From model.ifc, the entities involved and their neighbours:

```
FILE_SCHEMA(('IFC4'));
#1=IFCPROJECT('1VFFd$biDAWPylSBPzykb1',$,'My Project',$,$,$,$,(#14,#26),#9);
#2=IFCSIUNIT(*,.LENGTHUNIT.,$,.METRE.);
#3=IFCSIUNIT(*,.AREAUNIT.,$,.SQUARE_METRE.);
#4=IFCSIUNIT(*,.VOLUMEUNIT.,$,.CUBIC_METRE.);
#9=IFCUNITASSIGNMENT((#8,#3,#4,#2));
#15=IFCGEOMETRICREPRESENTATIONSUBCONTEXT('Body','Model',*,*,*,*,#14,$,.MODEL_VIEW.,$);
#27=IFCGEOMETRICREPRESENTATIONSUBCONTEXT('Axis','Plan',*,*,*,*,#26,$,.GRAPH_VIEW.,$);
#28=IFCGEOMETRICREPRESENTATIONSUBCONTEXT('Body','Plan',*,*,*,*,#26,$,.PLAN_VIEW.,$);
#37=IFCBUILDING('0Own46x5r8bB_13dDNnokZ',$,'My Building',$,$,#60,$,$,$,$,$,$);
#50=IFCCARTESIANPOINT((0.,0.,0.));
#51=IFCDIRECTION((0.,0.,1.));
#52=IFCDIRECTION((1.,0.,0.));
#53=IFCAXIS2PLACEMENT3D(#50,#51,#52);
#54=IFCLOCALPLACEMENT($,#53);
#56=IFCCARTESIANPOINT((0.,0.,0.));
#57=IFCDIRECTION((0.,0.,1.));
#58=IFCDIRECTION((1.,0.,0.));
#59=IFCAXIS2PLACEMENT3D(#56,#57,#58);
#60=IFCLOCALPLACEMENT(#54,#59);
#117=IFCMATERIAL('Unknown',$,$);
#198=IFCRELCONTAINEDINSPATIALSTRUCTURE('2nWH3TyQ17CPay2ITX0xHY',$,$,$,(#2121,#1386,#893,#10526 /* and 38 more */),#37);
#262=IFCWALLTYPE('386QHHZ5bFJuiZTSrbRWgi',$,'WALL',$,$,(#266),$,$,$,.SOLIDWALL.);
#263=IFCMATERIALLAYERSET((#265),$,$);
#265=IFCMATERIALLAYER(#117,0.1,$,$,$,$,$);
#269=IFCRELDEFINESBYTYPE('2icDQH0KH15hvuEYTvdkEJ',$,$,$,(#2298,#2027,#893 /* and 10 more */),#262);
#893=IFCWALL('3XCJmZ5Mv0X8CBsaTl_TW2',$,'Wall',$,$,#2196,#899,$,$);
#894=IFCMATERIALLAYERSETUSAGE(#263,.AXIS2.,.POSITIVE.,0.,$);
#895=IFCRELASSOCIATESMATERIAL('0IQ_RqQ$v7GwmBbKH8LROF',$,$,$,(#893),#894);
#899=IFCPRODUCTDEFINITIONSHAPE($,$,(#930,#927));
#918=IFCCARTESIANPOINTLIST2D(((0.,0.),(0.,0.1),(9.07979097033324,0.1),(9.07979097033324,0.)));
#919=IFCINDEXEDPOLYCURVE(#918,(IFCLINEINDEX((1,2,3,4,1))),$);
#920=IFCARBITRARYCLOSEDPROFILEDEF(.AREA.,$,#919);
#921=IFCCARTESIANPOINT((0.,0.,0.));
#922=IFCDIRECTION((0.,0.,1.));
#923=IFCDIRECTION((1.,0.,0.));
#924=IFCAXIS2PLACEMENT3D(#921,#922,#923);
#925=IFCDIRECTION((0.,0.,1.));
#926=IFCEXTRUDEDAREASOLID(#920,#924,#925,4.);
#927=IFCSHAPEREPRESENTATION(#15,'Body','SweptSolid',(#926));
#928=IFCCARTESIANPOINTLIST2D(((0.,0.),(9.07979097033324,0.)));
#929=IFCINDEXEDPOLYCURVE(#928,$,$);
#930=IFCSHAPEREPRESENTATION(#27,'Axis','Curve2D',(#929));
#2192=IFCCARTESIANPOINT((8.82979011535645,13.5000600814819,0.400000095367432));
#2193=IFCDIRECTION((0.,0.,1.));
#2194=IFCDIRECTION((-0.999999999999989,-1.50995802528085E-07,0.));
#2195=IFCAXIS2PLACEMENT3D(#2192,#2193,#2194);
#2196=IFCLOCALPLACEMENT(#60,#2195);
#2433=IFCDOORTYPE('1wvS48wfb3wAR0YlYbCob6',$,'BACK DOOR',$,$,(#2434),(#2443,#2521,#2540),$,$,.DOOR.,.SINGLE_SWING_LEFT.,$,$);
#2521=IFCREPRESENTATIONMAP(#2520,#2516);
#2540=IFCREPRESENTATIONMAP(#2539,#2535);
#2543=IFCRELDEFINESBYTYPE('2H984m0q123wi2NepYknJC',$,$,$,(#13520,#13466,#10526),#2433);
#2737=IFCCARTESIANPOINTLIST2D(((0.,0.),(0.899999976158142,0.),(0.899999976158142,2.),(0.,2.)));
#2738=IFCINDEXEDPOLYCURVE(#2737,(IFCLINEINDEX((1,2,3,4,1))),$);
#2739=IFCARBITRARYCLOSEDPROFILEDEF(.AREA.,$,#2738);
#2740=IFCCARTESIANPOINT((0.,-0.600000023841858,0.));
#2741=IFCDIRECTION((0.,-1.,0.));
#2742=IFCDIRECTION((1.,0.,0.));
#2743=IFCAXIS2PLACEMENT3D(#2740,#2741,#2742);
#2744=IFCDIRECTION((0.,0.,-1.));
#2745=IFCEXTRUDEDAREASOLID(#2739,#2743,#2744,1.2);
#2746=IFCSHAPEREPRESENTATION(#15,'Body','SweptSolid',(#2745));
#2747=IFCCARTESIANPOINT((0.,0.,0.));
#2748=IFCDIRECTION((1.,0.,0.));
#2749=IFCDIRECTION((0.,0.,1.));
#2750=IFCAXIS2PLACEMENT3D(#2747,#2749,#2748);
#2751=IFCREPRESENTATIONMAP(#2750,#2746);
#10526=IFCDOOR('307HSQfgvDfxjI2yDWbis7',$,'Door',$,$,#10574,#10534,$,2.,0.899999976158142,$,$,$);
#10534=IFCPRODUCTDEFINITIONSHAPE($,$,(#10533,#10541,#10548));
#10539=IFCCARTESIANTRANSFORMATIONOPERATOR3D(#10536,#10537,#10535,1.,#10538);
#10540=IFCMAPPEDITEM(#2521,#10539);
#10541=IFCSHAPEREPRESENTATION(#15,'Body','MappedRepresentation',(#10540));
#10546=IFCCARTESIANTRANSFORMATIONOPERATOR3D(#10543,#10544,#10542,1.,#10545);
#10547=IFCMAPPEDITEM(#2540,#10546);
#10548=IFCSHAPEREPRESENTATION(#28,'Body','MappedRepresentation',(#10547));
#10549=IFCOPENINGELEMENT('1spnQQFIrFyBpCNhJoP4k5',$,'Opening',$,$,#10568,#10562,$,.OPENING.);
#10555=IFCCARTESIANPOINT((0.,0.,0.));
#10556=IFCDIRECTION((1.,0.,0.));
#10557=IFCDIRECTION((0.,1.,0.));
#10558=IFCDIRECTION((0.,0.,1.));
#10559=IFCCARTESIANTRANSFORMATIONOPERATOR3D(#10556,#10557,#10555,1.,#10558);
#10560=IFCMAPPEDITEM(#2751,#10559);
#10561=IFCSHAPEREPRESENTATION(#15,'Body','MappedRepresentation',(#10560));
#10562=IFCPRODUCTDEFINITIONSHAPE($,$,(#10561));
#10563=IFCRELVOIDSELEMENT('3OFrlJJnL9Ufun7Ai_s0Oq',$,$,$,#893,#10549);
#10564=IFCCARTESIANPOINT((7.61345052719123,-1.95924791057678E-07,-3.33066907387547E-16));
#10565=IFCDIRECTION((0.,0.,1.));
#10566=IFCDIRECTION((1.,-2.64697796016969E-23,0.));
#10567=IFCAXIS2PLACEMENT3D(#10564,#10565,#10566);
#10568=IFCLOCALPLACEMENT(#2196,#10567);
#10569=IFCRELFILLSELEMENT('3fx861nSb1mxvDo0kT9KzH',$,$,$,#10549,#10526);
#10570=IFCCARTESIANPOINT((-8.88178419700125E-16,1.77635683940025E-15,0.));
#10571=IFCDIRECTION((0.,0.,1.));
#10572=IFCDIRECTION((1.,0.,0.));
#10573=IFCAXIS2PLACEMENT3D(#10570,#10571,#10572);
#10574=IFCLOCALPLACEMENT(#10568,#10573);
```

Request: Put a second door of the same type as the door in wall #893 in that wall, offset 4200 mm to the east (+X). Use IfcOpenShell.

```python
import ifcopenshell
import ifcopenshell.api.feature
import ifcopenshell.api.geometry
import ifcopenshell.api.root
import ifcopenshell.geom
import ifcopenshell.util.element
import ifcopenshell.util.placement
import ifcopenshell.util.shape
import ifcopenshell.util.unit

model = ifcopenshell.open("model.ifc")
unit_scale = ifcopenshell.util.unit.calculate_unit_scale(model)
settings = ifcopenshell.geom.settings()


def volume(element):
    """Net volume in cubic metres, openings subtracted."""
    shape = ifcopenshell.geom.create_shape(settings, element)
    return ifcopenshell.util.shape.get_volume(shape.geometry)


door = model.by_id(10526)
opening = door.FillsVoids[0].RelatingOpeningElement
wall = opening.VoidsElements[0].RelatingBuildingElement
before = volume(wall)
shift = ifcopenshell.util.placement.get_local_placement(wall.ObjectPlacement)[:3, 0] * -4.2 / unit_scale

# copy_class copies the void relationship, type, container and properties, but no geometry.
new_opening = ifcopenshell.api.root.copy_class(model, product=opening)
new_opening.Representation = ifcopenshell.util.element.copy_deep(
    model, opening.Representation, exclude=["IfcGeometricRepresentationContext", "IfcRepresentationMap"]
)
new_door = ifcopenshell.api.root.copy_class(model, product=door)
new_door.Representation = ifcopenshell.util.element.copy_deep(
    model, door.Representation, exclude=["IfcGeometricRepresentationContext", "IfcRepresentationMap"]
)
ifcopenshell.api.feature.add_filling(model, opening=new_opening, element=new_door)

for old, new in ((opening, new_opening), (door, new_door)):
    matrix = ifcopenshell.util.placement.get_local_placement(old.ObjectPlacement)
    matrix[:3, 3] += shift
    ifcopenshell.api.geometry.edit_object_placement(model, product=new, matrix=matrix, is_si=False)

after = volume(wall)

print(f"wall volume {before:.3f} -> {after:.3f} m3")

model.write("model_edited.ifc")
```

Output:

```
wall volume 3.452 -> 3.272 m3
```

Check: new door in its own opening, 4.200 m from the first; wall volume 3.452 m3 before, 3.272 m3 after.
